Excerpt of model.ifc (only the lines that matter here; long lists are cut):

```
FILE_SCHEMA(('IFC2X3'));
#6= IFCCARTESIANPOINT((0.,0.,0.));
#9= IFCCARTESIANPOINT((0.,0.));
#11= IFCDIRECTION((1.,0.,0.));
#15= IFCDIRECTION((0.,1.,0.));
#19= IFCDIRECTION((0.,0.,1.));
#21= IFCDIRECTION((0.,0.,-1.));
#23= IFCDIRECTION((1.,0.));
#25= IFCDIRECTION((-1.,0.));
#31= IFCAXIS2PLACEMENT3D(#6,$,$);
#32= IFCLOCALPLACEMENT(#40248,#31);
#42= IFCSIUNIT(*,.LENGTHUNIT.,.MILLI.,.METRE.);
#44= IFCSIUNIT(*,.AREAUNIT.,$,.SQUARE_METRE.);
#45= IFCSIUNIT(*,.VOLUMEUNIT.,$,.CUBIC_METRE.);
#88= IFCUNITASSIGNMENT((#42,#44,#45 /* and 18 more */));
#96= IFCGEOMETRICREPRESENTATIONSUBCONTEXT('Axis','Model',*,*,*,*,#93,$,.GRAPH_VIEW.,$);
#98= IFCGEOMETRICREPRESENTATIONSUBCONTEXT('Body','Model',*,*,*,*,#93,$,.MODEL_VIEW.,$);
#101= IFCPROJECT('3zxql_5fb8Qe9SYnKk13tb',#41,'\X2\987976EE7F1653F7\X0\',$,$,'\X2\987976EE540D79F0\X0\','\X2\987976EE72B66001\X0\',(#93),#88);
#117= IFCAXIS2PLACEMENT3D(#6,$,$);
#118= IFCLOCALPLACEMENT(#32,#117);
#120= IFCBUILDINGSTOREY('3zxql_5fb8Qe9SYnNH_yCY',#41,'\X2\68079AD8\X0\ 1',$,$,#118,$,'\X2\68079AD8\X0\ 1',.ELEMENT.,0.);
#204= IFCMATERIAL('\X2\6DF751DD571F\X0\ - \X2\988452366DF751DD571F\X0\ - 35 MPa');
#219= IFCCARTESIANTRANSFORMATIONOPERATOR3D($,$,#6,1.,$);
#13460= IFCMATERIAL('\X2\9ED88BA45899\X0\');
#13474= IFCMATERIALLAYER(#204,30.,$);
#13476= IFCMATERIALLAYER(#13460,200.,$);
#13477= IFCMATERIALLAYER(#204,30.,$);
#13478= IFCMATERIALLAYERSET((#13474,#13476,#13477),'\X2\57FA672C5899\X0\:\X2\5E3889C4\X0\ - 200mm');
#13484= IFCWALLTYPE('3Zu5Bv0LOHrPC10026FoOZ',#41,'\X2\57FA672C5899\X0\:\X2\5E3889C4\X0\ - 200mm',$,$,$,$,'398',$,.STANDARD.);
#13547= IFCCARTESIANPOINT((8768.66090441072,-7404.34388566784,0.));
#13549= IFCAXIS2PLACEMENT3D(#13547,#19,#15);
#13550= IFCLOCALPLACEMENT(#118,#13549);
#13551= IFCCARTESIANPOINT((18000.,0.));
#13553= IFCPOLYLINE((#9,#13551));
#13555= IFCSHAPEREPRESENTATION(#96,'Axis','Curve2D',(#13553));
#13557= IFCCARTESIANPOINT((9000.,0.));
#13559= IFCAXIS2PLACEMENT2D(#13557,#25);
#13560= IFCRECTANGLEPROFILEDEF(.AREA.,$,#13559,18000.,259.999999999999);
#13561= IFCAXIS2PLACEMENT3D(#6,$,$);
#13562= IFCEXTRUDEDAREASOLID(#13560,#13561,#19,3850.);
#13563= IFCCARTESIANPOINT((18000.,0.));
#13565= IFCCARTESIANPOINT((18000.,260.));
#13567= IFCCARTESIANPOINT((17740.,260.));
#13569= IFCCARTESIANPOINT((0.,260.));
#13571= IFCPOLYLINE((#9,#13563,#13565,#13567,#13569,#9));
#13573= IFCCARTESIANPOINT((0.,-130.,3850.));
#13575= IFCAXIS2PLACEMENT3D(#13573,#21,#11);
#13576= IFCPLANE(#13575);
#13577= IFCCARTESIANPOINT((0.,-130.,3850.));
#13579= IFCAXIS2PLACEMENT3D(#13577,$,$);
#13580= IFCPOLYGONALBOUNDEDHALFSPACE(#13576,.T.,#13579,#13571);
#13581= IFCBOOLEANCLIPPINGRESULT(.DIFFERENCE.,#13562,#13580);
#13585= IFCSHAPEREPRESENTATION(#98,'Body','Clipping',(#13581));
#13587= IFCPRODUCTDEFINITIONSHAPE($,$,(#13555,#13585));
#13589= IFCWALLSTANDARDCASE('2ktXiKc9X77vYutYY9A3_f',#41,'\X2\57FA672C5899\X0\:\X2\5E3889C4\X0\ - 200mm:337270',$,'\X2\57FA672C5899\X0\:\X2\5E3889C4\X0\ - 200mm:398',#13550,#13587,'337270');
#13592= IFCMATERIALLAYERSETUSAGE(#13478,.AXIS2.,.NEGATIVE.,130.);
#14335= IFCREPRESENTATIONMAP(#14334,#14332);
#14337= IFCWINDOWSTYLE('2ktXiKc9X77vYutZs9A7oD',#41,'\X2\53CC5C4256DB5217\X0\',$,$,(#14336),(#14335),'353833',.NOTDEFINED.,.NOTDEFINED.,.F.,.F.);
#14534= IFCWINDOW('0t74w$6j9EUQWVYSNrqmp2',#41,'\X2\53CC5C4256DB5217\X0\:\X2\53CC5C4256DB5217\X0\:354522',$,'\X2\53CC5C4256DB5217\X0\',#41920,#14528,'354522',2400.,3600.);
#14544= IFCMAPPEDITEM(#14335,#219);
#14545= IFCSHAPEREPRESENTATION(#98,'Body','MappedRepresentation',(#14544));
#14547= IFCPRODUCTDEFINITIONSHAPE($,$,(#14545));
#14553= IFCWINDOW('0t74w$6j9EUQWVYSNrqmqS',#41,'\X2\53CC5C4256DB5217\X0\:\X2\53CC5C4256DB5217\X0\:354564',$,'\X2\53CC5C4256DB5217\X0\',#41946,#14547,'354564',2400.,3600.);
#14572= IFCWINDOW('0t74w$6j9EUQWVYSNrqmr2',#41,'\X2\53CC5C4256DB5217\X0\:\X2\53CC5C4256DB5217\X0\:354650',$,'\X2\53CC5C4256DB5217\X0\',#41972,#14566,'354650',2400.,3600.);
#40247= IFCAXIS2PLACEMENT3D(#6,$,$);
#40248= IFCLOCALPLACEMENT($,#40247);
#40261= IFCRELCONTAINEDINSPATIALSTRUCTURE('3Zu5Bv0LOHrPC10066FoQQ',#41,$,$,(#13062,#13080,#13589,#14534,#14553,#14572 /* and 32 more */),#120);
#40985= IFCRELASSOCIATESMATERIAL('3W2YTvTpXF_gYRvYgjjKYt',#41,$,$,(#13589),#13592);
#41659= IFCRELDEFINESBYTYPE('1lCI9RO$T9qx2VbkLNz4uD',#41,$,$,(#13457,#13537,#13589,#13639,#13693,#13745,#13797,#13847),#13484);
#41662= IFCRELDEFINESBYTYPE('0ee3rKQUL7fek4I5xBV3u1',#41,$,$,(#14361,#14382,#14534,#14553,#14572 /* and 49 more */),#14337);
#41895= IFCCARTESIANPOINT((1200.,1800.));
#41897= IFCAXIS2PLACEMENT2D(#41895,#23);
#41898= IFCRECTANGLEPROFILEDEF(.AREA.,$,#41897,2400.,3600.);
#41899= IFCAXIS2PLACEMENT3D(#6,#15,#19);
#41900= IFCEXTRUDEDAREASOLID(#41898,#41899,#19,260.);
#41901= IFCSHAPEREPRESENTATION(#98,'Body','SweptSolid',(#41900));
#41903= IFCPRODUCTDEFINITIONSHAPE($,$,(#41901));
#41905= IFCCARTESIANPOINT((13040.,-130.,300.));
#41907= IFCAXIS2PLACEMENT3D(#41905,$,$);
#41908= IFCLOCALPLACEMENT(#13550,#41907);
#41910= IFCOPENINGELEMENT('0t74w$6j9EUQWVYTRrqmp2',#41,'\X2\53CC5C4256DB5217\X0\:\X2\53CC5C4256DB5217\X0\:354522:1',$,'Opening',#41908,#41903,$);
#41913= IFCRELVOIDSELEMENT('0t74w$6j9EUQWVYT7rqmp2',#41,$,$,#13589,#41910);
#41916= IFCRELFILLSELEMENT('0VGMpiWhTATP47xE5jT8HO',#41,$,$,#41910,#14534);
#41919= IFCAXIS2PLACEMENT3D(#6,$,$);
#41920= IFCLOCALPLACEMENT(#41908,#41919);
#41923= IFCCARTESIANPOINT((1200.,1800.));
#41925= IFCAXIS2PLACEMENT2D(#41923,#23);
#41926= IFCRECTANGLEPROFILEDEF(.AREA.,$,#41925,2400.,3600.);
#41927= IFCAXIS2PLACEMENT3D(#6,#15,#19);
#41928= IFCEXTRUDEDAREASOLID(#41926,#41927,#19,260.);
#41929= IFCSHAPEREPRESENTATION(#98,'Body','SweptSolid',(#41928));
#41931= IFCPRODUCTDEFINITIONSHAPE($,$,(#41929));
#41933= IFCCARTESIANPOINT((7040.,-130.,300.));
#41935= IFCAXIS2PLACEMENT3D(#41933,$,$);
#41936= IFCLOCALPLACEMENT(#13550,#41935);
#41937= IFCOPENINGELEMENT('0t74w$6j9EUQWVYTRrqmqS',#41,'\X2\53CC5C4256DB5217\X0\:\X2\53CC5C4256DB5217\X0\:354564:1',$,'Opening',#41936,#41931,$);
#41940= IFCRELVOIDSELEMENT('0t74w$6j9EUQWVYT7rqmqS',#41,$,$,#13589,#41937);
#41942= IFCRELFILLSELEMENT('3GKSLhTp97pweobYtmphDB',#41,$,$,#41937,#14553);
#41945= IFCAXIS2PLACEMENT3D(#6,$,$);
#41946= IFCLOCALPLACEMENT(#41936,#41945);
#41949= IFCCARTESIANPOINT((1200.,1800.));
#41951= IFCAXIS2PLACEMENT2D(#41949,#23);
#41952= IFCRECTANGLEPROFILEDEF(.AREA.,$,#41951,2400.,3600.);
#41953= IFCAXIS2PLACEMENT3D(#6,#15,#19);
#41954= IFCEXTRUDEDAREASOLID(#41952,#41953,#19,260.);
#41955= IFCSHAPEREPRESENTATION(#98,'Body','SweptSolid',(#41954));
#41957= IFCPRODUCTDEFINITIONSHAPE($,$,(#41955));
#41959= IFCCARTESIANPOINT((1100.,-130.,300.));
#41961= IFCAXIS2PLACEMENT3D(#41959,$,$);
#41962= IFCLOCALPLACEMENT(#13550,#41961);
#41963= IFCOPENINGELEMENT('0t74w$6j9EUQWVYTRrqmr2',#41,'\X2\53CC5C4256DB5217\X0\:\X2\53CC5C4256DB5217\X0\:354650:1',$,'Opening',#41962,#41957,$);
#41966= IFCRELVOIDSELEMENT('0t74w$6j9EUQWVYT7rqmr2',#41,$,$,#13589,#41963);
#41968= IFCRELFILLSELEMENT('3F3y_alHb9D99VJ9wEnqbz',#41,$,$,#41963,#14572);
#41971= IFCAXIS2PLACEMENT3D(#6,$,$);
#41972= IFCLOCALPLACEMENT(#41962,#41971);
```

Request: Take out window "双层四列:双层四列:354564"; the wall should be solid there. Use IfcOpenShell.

```python
import ifcopenshell
import ifcopenshell.api.feature
import ifcopenshell.api.root
import ifcopenshell.geom
import ifcopenshell.util.shape

model = ifcopenshell.open("model.ifc")
settings = ifcopenshell.geom.settings()


def volume(element):
    """Net volume in cubic metres, openings subtracted."""
    shape = ifcopenshell.geom.create_shape(settings, element)
    return ifcopenshell.util.shape.get_volume(shape.geometry)


window = model.by_guid("0t74w$6j9EUQWVYSNrqmqS")
opening = window.FillsVoids[0].RelatingOpeningElement
wall = opening.VoidsElements[0].RelatingBuildingElement
before = volume(wall)

ifcopenshell.api.root.remove_product(model, product=window)
ifcopenshell.api.feature.remove_feature(model, feature=opening)

after = volume(wall)

print(f"wall volume {before:.3f} -> {after:.3f} m3")

model.write("model_v2.ifc")
```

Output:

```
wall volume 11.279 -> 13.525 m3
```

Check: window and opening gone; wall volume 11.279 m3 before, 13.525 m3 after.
